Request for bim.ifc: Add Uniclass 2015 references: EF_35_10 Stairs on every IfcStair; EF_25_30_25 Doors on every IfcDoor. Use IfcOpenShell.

First a look at what the model holds.

```python
import ifcopenshell

model = ifcopenshell.open("bim.ifc")
print(model.schema)
print("classifications:", [c.Name for c in model.by_type("IfcClassification")])
for ifc_class in ("IfcDoor", "IfcRoof", "IfcStair", "IfcWall", "IfcWindow"):
    print(ifc_class, len(model.by_type(ifc_class)))
```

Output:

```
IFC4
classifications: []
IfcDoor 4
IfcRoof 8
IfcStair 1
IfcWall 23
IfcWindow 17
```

```python
import ifcopenshell
import ifcopenshell.api.classification

model = ifcopenshell.open("bim.ifc")

system = ifcopenshell.api.classification.add_classification(model, classification="Uniclass 2015")

codes = {
    "IfcStair": ("EF_35_10", "Stairs"),
    "IfcDoor": ("EF_25_30_25", "Doors"),
}
for ifc_class, (code, name) in codes.items():
    products = model.by_type(ifc_class)
    ifcopenshell.api.classification.add_reference(
        model, products=products, classification=system, identification=code, name=name
    )
    print(code, len(products))

model.write("bim-out.ifc")
```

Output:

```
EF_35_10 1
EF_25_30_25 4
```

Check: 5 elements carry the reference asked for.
